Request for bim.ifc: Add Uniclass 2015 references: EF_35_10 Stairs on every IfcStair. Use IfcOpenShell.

First a look at what the model holds.

```python
import ifcopenshell

model = ifcopenshell.open("bim.ifc")
print(model.schema)
print("classifications:", [c.Name for c in model.by_type("IfcClassification")])
for ifc_class in ("IfcDoor", "IfcRoof", "IfcStair", "IfcWall", "IfcWindow"):
    print(ifc_class, len(model.by_type(ifc_class)))
```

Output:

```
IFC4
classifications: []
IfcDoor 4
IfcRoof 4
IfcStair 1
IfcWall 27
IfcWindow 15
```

```python
import ifcopenshell
import ifcopenshell.api.classification

model = ifcopenshell.open("bim.ifc")

system = ifcopenshell.api.classification.add_classification(model, classification="Uniclass 2015")

codes = {
    "IfcStair": ("EF_35_10", "Stairs"),
}
for ifc_class, (code, name) in codes.items():
    products = model.by_type(ifc_class)
    ifcopenshell.api.classification.add_reference(
        model, products=products, classification=system, identification=code, name=name
    )
    print(code, len(products))

model.write("bim-out.ifc")
```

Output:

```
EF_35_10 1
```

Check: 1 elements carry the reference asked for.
